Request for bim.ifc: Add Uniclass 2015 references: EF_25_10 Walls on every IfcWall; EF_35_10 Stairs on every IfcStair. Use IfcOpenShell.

First a look at what the model holds.

```python
import ifcopenshell

model = ifcopenshell.open("bim.ifc")
print(model.schema)
print("classifications:", [c.Name for c in model.by_type("IfcClassification")])
for ifc_class in ("IfcDoor", "IfcRoof", "IfcStair", "IfcWall", "IfcWindow"):
    print(ifc_class, len(model.by_type(ifc_class)))
```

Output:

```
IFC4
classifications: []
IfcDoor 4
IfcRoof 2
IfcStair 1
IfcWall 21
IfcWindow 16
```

```python
import ifcopenshell
import ifcopenshell.api.classification

model = ifcopenshell.open("bim.ifc")

system = ifcopenshell.api.classification.add_classification(model, classification="Uniclass 2015")

codes = {
    "IfcWall": ("EF_25_10", "Walls"),
    "IfcStair": ("EF_35_10", "Stairs"),
}
for ifc_class, (code, name) in codes.items():
    products = model.by_type(ifc_class)
    ifcopenshell.api.classification.add_reference(
        model, products=products, classification=system, identification=code, name=name
    )
    print(code, len(products))

model.write("bim-out.ifc")
```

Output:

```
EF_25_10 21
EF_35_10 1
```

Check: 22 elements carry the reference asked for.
